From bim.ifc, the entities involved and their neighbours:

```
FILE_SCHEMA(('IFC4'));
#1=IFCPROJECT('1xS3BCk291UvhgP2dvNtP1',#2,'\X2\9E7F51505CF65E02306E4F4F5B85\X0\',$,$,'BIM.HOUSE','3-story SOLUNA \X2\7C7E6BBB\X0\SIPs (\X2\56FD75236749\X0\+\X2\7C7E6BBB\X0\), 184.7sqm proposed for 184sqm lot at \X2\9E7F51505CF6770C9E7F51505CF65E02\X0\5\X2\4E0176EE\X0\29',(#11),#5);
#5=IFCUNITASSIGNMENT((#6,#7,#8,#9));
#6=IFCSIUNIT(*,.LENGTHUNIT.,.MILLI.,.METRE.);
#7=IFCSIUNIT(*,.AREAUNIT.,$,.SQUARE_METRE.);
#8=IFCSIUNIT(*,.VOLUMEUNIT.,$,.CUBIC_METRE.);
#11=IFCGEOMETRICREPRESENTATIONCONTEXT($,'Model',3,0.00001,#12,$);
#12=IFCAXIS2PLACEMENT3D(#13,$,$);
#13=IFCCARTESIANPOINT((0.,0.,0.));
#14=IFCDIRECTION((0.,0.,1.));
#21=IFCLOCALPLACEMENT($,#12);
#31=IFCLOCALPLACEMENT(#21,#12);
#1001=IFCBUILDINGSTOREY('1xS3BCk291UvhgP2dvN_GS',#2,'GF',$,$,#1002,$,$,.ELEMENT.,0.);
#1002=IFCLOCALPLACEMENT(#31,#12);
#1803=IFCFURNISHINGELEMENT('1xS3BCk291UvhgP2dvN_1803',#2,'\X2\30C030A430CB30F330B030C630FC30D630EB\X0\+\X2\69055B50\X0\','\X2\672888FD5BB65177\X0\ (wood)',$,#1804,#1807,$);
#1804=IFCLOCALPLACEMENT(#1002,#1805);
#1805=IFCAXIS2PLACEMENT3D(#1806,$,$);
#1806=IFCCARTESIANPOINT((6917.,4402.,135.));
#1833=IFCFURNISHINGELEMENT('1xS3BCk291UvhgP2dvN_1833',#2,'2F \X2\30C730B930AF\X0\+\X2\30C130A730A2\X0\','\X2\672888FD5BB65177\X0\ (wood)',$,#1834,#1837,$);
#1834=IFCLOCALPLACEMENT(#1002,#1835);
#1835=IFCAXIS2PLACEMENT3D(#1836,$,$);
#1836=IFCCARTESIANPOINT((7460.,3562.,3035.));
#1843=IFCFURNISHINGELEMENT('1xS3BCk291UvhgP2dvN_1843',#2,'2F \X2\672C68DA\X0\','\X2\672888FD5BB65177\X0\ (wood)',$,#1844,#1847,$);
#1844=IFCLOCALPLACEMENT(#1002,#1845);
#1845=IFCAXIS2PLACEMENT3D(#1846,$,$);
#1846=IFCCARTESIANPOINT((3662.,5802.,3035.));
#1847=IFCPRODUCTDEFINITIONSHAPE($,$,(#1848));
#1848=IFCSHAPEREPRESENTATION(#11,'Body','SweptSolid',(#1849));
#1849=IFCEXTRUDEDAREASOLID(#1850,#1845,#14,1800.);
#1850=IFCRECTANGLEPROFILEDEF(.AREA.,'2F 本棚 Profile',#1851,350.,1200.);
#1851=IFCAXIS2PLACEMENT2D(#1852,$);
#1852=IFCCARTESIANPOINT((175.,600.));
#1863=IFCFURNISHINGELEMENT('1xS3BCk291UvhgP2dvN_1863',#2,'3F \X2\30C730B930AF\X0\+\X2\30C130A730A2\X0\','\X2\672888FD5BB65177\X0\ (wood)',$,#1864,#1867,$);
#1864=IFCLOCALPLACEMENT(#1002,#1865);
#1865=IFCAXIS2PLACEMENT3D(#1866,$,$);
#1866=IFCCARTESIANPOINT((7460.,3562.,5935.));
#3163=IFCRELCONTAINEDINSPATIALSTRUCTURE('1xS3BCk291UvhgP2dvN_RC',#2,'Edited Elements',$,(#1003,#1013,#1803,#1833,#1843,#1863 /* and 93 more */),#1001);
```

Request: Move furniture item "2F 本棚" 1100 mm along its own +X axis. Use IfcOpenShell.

```python
import ifcopenshell
import ifcopenshell.api.geometry
import ifcopenshell.util.placement
import ifcopenshell.util.unit

model = ifcopenshell.open("bim.ifc")
unit_scale = ifcopenshell.util.unit.calculate_unit_scale(model)

item = model.by_guid("1xS3BCk291UvhgP2dvN_1843")
matrix = ifcopenshell.util.placement.get_local_placement(item.ObjectPlacement)
matrix[:3, 3] += matrix[:3, 0] * 1.1 / unit_scale
ifcopenshell.api.geometry.edit_object_placement(model, product=item, matrix=matrix, is_si=False)

print(ifcopenshell.util.placement.get_local_placement(item.ObjectPlacement).round(3) + 0.0)

model.write("bim_rev.ifc")
```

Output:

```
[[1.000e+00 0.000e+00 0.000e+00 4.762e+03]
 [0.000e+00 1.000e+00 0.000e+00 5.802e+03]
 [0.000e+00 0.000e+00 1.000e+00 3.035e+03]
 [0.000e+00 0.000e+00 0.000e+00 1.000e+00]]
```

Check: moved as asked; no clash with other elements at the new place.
